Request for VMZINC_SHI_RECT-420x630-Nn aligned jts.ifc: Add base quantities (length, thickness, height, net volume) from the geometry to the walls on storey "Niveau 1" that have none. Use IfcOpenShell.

First a look at what the model holds.

```python
import ifcopenshell
import ifcopenshell.util.element
import ifcopenshell.util.unit

model = ifcopenshell.open("VMZINC_SHI_RECT-420x630-Nn aligned jts.ifc")
print(model.schema)
for unit_type in ("LENGTHUNIT", "AREAUNIT", "VOLUMEUNIT"):
    print(unit_type, ifcopenshell.util.unit.calculate_unit_scale(model, unit_type))
storey = next(s for s in model.by_type("IfcBuildingStorey") if s.Name == "Niveau 1")
walls = [e for e in ifcopenshell.util.element.get_decomposition(storey) if e.is_a("IfcWall")]
for e in sorted(walls, key=lambda e: e.id()):
    print(e.id(), e.is_a(), e.Name, list(ifcopenshell.util.element.get_psets(e, qtos_only=True)), sep=" | ")
```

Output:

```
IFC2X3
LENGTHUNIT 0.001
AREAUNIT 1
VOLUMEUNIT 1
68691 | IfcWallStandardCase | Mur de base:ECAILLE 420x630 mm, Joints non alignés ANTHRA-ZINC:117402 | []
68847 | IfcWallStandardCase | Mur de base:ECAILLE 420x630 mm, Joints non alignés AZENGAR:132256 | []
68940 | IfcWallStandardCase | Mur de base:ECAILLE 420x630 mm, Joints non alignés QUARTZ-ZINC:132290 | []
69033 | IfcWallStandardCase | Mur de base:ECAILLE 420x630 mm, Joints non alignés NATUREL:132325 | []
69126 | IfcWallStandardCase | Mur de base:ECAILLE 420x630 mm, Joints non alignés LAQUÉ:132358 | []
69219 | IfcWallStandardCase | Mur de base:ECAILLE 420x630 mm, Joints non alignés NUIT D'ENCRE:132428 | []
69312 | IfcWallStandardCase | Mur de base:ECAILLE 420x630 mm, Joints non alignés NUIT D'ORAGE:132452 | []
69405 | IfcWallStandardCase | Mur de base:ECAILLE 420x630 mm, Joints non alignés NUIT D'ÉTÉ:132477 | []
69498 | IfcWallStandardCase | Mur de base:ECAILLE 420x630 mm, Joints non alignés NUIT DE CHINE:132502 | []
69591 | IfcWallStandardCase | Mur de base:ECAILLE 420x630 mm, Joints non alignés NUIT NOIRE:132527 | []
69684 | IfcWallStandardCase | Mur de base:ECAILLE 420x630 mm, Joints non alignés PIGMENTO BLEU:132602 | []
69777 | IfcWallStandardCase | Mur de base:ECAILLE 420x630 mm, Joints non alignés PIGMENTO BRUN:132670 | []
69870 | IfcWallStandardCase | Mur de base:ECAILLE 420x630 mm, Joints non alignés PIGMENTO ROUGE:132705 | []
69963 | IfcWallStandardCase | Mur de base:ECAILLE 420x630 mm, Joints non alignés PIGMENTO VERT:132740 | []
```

```python
import ifcopenshell
import ifcopenshell.api.pset
import ifcopenshell.geom
import ifcopenshell.util.element
import ifcopenshell.util.shape
import ifcopenshell.util.unit

model = ifcopenshell.open("VMZINC_SHI_RECT-420x630-Nn aligned jts.ifc")
unit_scale = ifcopenshell.util.unit.calculate_unit_scale(model)
volume_scale = ifcopenshell.util.unit.calculate_unit_scale(model, "VOLUMEUNIT")
settings = ifcopenshell.geom.settings()

storey = next(s for s in model.by_type("IfcBuildingStorey") if s.Name == "Niveau 1")
walls = [e for e in ifcopenshell.util.element.get_decomposition(storey) if e.is_a("IfcWall")]

for e in sorted(walls, key=lambda e: e.id()):
    if ifcopenshell.util.element.get_psets(e, qtos_only=True, should_inherit=False):
        continue
    # Geometry comes back in metres, in the element's own axes.
    shape = ifcopenshell.geom.create_shape(settings, e)
    values = {
        "Length": ifcopenshell.util.shape.get_x(shape.geometry) / unit_scale,
        "Width": ifcopenshell.util.shape.get_y(shape.geometry) / unit_scale,
        "Height": ifcopenshell.util.shape.get_z(shape.geometry) / unit_scale,
        "NetVolume": ifcopenshell.util.shape.get_volume(shape.geometry) / volume_scale,
    }
    qto = ifcopenshell.api.pset.add_qto(model, product=e, name="BaseQuantities")
    ifcopenshell.api.pset.edit_qto(model, qto=qto, properties=values)
    print(e.id(), {k: round(v, 3) for k, v in values.items()})

model.write("VMZINC_SHI_RECT-420x630-Nn aligned jts_rev.ifc")
```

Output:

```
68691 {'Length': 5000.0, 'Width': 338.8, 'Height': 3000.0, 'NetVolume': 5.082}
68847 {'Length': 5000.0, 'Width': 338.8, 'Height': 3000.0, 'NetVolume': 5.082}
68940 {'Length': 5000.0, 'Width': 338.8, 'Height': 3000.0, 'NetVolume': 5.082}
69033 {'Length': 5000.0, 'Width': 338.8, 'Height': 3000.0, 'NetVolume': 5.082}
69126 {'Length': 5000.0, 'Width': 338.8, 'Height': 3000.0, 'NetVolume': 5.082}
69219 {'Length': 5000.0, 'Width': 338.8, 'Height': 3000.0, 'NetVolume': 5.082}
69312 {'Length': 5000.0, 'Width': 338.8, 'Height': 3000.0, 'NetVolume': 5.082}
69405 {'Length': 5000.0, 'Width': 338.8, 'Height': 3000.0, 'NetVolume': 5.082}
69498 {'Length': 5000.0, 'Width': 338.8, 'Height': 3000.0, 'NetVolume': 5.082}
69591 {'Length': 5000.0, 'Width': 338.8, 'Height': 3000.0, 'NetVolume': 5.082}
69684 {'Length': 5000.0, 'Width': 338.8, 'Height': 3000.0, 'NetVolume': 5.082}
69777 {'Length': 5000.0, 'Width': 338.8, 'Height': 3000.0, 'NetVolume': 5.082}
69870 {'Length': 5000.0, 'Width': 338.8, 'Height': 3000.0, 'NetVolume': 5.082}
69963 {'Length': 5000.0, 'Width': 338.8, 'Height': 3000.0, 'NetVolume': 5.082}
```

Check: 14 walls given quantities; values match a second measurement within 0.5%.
